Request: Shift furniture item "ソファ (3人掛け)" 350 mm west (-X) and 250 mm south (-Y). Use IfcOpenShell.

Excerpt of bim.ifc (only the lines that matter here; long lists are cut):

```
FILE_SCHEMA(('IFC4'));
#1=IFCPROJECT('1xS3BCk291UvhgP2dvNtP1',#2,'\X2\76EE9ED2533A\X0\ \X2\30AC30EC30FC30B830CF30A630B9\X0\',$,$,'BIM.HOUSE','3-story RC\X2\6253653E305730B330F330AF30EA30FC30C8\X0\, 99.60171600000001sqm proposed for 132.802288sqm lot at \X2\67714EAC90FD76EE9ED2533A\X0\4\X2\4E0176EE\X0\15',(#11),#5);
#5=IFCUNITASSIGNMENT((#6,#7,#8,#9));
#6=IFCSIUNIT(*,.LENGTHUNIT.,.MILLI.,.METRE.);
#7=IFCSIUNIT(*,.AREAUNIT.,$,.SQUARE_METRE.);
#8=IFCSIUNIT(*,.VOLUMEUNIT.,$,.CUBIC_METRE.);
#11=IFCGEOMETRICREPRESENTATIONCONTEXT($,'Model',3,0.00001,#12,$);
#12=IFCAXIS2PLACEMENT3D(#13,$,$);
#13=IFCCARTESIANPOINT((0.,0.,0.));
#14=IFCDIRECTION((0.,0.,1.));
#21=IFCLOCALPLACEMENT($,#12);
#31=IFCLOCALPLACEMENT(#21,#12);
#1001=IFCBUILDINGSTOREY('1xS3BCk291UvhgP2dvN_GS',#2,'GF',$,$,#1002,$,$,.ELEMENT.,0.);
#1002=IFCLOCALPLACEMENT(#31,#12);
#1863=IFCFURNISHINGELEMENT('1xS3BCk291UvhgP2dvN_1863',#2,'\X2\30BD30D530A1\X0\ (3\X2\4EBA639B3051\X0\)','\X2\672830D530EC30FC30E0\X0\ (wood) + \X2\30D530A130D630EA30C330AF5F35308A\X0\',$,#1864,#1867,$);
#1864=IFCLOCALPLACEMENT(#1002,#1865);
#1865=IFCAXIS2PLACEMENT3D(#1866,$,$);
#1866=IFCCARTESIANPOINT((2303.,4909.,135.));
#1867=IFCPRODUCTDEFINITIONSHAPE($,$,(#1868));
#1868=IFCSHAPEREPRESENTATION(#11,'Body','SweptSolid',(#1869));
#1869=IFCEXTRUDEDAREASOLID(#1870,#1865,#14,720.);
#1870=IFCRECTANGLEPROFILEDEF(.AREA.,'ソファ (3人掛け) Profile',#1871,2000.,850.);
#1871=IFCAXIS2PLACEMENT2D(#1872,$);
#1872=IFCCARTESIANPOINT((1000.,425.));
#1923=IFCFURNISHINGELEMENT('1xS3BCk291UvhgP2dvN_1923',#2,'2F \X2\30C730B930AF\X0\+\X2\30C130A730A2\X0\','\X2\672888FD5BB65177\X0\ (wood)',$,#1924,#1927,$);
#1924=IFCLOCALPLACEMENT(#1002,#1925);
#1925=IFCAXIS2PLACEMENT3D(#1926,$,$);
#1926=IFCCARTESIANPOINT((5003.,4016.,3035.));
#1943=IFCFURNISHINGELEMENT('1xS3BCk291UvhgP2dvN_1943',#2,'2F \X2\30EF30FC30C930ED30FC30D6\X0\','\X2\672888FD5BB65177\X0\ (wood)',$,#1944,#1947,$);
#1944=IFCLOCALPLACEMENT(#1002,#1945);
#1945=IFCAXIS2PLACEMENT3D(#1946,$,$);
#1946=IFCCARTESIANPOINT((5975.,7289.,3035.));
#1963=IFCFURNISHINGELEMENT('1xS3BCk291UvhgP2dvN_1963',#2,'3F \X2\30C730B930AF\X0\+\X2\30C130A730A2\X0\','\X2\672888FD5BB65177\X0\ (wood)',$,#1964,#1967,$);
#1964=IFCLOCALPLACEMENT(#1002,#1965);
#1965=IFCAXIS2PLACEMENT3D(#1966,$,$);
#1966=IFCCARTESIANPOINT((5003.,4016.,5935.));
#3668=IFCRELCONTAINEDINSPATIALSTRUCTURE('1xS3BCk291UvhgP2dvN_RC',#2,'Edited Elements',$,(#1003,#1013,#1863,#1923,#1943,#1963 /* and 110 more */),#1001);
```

```python
import ifcopenshell
import ifcopenshell.api.geometry
import ifcopenshell.util.placement
import ifcopenshell.util.unit

model = ifcopenshell.open("bim.ifc")
unit_scale = ifcopenshell.util.unit.calculate_unit_scale(model)

item = model.by_guid("1xS3BCk291UvhgP2dvN_1863")
matrix = ifcopenshell.util.placement.get_local_placement(item.ObjectPlacement)
matrix[0, 3] -= 0.35 / unit_scale
matrix[1, 3] -= 0.25 / unit_scale
ifcopenshell.api.geometry.edit_object_placement(model, product=item, matrix=matrix, is_si=False)

print(ifcopenshell.util.placement.get_local_placement(item.ObjectPlacement).round(3) + 0.0)

model.write("bim_updated.ifc")
```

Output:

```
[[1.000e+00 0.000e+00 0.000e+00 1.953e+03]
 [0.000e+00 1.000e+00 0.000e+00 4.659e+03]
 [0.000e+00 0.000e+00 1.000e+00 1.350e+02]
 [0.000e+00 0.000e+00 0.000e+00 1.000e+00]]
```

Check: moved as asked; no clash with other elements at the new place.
